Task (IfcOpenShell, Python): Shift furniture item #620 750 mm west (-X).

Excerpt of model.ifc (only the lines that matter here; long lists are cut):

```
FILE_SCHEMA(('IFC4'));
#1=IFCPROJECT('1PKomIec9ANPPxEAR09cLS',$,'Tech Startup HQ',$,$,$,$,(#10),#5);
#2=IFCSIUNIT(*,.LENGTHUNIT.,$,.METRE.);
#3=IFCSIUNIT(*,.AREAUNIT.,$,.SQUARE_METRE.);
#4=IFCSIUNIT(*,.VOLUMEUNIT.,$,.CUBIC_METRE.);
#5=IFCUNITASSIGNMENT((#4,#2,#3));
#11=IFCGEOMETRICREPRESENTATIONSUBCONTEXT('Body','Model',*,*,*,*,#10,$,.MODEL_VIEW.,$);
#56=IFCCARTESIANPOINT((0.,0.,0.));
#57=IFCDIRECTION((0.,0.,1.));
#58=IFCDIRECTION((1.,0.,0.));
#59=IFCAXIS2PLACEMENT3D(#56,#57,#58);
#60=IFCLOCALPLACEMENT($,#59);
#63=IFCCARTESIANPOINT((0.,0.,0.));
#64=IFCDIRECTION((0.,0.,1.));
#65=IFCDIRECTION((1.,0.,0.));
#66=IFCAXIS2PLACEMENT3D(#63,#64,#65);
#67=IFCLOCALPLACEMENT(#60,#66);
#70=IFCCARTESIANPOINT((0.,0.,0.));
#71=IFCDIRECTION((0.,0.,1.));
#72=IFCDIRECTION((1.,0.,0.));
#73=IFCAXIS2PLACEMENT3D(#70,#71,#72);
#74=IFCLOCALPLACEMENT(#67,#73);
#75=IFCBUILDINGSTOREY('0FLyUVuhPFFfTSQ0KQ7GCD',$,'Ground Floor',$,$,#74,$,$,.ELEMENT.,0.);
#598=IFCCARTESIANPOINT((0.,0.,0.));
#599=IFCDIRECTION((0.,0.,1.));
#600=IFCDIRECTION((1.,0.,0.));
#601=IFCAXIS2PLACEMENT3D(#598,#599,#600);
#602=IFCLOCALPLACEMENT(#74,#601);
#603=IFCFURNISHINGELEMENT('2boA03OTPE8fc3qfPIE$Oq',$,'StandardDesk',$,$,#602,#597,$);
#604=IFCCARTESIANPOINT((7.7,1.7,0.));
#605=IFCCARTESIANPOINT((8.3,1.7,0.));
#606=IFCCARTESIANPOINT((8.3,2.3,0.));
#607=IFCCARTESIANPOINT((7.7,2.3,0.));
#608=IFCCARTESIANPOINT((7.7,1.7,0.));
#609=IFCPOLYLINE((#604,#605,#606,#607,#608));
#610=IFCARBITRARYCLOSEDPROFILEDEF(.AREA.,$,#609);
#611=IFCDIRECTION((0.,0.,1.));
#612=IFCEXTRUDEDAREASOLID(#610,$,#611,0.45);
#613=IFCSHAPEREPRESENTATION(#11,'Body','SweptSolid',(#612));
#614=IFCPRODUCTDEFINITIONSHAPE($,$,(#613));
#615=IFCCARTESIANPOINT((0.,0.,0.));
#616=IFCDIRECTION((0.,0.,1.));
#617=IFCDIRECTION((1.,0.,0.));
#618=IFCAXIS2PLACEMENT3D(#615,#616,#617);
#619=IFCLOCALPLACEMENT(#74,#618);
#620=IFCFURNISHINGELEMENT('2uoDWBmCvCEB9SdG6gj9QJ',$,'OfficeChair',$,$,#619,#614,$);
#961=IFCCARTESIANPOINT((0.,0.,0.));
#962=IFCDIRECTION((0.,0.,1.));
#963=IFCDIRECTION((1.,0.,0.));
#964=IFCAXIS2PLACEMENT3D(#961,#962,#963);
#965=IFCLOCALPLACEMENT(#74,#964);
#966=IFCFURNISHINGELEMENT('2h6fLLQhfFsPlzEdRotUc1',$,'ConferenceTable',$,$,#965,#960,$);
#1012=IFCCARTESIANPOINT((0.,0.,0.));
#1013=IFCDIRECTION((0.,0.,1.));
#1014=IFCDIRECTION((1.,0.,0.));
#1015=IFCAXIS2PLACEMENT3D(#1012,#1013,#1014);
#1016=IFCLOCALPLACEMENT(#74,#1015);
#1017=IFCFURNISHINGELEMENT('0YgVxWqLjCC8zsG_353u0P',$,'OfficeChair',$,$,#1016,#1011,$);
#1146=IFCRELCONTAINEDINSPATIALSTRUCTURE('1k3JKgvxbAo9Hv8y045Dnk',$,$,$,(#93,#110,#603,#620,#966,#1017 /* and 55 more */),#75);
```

```python
import ifcopenshell
import ifcopenshell.api.geometry
import ifcopenshell.util.placement
import ifcopenshell.util.unit

model = ifcopenshell.open("model.ifc")
unit_scale = ifcopenshell.util.unit.calculate_unit_scale(model)

item = model.by_guid("2uoDWBmCvCEB9SdG6gj9QJ")
matrix = ifcopenshell.util.placement.get_local_placement(item.ObjectPlacement)
matrix[0, 3] -= 0.75 / unit_scale
ifcopenshell.api.geometry.edit_object_placement(model, product=item, matrix=matrix, is_si=False)

print(ifcopenshell.util.placement.get_local_placement(item.ObjectPlacement).round(3) + 0.0)

model.write("model_v2.ifc")
```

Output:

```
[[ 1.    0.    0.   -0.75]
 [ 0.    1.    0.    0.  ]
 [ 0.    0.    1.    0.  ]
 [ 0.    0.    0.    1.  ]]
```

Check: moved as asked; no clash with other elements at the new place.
